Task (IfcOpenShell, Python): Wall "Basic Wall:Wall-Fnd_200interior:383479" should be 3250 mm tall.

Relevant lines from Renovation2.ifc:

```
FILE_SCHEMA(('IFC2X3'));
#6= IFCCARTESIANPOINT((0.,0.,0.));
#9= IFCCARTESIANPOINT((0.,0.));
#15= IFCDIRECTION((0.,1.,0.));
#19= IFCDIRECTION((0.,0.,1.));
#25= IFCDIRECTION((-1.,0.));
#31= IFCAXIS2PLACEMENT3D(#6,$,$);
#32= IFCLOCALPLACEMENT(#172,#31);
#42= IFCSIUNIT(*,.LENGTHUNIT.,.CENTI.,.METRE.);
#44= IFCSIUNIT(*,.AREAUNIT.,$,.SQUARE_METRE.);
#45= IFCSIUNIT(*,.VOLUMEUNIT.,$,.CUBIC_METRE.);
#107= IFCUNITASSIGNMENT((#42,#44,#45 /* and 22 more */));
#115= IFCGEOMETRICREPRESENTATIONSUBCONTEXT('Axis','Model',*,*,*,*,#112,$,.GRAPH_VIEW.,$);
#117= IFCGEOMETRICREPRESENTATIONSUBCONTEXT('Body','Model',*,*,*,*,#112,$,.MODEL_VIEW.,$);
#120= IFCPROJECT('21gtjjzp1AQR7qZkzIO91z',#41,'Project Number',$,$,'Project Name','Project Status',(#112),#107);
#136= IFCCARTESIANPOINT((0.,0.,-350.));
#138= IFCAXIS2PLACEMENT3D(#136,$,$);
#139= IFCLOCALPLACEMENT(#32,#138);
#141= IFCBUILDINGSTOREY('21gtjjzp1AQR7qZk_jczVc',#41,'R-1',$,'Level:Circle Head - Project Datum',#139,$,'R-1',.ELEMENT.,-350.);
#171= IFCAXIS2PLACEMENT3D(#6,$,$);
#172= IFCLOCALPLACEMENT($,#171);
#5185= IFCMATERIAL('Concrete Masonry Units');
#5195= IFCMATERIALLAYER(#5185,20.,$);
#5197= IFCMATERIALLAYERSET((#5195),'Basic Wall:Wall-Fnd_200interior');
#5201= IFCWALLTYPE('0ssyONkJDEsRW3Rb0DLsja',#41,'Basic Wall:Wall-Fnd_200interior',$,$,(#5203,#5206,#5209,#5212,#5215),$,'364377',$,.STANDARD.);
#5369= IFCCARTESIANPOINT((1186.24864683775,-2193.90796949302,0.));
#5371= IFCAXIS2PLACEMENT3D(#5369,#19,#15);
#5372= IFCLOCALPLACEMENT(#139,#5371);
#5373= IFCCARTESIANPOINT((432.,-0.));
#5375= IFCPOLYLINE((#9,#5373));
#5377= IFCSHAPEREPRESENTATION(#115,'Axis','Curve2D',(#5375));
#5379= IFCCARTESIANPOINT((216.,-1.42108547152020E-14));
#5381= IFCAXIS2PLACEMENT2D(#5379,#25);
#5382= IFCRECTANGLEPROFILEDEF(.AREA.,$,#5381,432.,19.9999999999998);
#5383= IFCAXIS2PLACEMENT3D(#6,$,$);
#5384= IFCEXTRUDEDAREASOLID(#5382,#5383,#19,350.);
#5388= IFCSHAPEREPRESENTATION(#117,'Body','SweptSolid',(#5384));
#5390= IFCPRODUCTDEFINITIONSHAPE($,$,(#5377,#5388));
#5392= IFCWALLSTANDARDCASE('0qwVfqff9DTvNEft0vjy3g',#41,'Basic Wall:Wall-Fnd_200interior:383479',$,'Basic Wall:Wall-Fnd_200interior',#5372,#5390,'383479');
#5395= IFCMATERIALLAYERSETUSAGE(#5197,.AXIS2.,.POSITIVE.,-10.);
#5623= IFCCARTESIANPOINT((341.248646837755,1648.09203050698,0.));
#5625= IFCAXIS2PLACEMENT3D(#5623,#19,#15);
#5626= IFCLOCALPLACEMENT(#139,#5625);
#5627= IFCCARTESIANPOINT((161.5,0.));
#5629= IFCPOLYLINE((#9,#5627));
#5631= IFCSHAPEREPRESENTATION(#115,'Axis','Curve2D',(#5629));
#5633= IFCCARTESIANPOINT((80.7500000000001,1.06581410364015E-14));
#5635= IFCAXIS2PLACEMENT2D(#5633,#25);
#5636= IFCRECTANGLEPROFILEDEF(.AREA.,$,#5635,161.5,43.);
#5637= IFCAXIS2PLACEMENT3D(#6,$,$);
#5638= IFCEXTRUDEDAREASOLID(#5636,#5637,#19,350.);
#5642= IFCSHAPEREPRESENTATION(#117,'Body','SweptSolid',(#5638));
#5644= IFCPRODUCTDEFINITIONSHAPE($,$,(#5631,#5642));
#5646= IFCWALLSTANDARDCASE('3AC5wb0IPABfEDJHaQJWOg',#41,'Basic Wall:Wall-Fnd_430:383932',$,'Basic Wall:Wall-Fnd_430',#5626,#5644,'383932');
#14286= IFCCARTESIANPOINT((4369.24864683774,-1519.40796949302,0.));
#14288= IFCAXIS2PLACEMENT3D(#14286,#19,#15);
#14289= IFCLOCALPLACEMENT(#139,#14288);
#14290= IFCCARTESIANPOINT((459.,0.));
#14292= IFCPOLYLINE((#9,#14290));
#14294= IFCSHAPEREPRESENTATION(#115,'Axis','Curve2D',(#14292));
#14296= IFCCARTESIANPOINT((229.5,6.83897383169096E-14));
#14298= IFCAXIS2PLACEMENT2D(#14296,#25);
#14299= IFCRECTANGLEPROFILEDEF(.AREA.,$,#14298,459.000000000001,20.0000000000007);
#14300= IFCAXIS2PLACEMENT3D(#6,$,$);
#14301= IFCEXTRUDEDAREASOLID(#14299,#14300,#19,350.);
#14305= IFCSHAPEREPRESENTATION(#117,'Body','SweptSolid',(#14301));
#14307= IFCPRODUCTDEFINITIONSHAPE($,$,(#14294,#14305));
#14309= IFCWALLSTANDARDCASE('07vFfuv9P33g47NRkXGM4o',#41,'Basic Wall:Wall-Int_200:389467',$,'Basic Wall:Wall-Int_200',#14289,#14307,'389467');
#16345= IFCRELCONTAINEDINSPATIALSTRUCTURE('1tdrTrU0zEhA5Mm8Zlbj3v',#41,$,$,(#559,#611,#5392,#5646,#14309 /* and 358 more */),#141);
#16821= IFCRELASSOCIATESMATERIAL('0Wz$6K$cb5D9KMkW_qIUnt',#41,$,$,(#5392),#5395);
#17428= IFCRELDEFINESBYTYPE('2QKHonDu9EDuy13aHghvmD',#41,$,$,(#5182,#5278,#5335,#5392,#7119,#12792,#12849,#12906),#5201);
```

```python
import ifcopenshell
import ifcopenshell.geom
import ifcopenshell.util.representation
import ifcopenshell.util.shape
import ifcopenshell.util.unit

model = ifcopenshell.open("Renovation2.ifc")
unit_scale = ifcopenshell.util.unit.calculate_unit_scale(model)
settings = ifcopenshell.geom.settings()


def volume(element):
    """Net volume in cubic metres, openings subtracted."""
    shape = ifcopenshell.geom.create_shape(settings, element)
    return ifcopenshell.util.shape.get_volume(shape.geometry)


wall = model.by_guid("0qwVfqff9DTvNEft0vjy3g")
before = volume(wall)

body = ifcopenshell.util.representation.get_representation(wall, "Model", "Body")
solid = body.Items[0]
old_height = solid.Depth
solid.Depth = 3.25 / unit_scale
after = volume(wall)

print(f"height {old_height:g} -> {solid.Depth:g}, volume {before:.3f} -> {after:.3f} m3")

model.write("Renovation2_edited.ifc")
```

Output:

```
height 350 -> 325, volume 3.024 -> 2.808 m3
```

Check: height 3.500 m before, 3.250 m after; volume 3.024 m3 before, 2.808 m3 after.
